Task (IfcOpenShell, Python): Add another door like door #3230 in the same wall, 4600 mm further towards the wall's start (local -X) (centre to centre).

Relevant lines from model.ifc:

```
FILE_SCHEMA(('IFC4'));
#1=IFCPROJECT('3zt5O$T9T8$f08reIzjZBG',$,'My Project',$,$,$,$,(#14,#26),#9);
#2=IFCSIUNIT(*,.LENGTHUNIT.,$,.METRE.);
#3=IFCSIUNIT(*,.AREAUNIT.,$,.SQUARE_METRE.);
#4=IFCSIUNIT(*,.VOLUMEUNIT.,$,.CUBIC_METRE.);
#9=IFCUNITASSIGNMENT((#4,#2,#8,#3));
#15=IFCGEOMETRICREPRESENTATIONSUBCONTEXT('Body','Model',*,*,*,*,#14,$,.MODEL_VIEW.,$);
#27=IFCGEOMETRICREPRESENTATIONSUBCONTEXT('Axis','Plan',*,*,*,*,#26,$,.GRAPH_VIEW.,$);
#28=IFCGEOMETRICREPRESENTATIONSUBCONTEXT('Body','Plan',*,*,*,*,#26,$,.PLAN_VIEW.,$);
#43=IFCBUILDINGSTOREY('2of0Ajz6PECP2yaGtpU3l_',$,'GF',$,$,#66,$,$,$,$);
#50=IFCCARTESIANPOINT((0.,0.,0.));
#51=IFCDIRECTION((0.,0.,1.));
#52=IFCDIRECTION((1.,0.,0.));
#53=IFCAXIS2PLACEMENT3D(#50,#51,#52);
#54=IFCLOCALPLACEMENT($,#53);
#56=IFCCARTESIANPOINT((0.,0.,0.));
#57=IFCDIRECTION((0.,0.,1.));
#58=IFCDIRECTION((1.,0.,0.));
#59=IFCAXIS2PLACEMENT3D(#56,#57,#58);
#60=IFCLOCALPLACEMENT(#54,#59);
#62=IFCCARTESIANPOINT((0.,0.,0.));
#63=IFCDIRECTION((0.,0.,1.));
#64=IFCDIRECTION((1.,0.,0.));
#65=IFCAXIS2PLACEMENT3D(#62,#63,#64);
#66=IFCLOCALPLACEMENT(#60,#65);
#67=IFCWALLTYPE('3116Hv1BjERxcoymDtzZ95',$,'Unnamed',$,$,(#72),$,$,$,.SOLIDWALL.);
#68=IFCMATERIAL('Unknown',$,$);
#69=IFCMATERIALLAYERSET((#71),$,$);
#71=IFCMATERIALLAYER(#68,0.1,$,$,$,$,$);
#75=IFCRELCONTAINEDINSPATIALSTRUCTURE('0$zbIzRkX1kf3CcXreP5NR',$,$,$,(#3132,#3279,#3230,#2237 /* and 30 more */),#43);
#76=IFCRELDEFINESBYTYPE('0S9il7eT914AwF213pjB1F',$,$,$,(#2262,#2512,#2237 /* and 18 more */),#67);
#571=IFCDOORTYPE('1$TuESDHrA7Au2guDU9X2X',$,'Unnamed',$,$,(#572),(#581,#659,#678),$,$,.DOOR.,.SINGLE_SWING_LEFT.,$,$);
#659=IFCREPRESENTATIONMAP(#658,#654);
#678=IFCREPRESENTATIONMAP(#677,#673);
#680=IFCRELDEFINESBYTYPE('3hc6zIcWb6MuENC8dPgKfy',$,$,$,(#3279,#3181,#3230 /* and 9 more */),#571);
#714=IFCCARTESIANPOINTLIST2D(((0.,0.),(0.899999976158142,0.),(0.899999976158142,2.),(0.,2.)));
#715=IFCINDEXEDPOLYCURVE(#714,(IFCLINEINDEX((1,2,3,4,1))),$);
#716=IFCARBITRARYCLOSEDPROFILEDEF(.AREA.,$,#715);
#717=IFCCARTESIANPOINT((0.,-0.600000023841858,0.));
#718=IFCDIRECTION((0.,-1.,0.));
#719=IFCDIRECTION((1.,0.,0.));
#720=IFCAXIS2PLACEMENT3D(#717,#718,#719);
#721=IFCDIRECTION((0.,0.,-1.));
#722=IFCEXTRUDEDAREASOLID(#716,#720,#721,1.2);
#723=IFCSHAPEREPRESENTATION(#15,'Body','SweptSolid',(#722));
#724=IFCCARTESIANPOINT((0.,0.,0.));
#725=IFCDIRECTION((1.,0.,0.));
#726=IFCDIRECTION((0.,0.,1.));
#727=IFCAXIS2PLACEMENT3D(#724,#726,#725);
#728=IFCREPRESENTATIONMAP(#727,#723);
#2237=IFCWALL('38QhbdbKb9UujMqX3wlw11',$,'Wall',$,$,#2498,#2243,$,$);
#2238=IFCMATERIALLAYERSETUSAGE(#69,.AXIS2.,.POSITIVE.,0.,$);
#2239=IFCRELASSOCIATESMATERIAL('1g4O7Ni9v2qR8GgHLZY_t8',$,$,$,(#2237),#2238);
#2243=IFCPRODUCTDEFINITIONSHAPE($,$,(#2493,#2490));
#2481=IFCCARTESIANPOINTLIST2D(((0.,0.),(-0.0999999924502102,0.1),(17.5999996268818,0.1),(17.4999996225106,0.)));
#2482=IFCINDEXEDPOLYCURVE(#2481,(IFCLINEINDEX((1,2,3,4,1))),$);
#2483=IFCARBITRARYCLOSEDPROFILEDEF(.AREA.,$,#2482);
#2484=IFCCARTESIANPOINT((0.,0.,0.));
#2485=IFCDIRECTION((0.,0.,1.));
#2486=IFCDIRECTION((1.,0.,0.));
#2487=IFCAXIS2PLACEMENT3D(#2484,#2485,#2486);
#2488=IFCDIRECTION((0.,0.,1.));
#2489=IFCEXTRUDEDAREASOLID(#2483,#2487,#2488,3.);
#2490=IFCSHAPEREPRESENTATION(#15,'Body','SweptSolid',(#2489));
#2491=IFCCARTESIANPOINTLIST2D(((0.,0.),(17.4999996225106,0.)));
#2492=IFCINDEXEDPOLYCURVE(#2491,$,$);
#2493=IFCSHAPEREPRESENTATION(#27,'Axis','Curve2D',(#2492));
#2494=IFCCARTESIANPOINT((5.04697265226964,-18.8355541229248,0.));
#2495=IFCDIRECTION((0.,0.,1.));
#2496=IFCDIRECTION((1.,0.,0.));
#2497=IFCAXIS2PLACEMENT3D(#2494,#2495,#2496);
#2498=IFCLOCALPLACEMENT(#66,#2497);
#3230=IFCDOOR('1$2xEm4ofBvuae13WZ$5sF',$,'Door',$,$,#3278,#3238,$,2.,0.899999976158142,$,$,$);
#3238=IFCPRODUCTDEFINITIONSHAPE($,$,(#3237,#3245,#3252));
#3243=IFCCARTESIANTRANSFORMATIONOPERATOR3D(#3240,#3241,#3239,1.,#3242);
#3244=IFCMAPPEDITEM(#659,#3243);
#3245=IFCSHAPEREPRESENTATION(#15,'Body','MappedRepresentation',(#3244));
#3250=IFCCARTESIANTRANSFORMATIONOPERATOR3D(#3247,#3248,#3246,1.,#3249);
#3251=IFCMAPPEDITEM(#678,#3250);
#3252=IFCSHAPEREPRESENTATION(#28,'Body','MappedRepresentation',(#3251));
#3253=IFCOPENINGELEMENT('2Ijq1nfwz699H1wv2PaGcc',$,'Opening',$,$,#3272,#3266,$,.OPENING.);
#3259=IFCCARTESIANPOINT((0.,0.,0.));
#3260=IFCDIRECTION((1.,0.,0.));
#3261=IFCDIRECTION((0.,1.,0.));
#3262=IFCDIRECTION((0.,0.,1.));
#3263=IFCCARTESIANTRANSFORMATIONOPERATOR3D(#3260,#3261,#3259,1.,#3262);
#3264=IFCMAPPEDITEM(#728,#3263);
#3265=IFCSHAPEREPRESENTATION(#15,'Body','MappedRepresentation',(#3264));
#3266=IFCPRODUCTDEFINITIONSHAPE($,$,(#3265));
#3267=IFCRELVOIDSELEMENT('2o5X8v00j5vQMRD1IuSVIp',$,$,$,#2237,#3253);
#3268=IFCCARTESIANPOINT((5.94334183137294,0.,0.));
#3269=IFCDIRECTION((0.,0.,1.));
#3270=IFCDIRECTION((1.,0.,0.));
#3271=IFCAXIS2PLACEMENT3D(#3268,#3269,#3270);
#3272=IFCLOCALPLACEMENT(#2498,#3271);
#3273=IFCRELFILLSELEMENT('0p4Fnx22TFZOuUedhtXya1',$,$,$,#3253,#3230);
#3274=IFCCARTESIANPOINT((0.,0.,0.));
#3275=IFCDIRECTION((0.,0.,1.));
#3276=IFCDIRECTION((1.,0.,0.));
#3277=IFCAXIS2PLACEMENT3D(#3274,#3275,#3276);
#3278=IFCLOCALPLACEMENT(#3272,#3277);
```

```python
import ifcopenshell
import ifcopenshell.api.feature
import ifcopenshell.api.geometry
import ifcopenshell.api.root
import ifcopenshell.geom
import ifcopenshell.util.element
import ifcopenshell.util.placement
import ifcopenshell.util.shape
import ifcopenshell.util.unit

model = ifcopenshell.open("model.ifc")
unit_scale = ifcopenshell.util.unit.calculate_unit_scale(model)
settings = ifcopenshell.geom.settings()


def volume(element):
    """Net volume in cubic metres, openings subtracted."""
    shape = ifcopenshell.geom.create_shape(settings, element)
    return ifcopenshell.util.shape.get_volume(shape.geometry)


door = model.by_guid("1$2xEm4ofBvuae13WZ$5sF")
opening = door.FillsVoids[0].RelatingOpeningElement
wall = opening.VoidsElements[0].RelatingBuildingElement
before = volume(wall)
shift = ifcopenshell.util.placement.get_local_placement(wall.ObjectPlacement)[:3, 0] * -4.6 / unit_scale

# copy_class copies the void relationship, type, container and properties, but no geometry.
new_opening = ifcopenshell.api.root.copy_class(model, product=opening)
new_opening.Representation = ifcopenshell.util.element.copy_deep(
    model, opening.Representation, exclude=["IfcGeometricRepresentationContext", "IfcRepresentationMap"]
)
new_door = ifcopenshell.api.root.copy_class(model, product=door)
new_door.Representation = ifcopenshell.util.element.copy_deep(
    model, door.Representation, exclude=["IfcGeometricRepresentationContext", "IfcRepresentationMap"]
)
ifcopenshell.api.feature.add_filling(model, opening=new_opening, element=new_door)

for old, new in ((opening, new_opening), (door, new_door)):
    matrix = ifcopenshell.util.placement.get_local_placement(old.ObjectPlacement)
    matrix[:3, 3] += shift
    ifcopenshell.api.geometry.edit_object_placement(model, product=new, matrix=matrix, is_si=False)

after = volume(wall)

print(f"wall volume {before:.3f} -> {after:.3f} m3")

model.write("model_rev.ifc")
```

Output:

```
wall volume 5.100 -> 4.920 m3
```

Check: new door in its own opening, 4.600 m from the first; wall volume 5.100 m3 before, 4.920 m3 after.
